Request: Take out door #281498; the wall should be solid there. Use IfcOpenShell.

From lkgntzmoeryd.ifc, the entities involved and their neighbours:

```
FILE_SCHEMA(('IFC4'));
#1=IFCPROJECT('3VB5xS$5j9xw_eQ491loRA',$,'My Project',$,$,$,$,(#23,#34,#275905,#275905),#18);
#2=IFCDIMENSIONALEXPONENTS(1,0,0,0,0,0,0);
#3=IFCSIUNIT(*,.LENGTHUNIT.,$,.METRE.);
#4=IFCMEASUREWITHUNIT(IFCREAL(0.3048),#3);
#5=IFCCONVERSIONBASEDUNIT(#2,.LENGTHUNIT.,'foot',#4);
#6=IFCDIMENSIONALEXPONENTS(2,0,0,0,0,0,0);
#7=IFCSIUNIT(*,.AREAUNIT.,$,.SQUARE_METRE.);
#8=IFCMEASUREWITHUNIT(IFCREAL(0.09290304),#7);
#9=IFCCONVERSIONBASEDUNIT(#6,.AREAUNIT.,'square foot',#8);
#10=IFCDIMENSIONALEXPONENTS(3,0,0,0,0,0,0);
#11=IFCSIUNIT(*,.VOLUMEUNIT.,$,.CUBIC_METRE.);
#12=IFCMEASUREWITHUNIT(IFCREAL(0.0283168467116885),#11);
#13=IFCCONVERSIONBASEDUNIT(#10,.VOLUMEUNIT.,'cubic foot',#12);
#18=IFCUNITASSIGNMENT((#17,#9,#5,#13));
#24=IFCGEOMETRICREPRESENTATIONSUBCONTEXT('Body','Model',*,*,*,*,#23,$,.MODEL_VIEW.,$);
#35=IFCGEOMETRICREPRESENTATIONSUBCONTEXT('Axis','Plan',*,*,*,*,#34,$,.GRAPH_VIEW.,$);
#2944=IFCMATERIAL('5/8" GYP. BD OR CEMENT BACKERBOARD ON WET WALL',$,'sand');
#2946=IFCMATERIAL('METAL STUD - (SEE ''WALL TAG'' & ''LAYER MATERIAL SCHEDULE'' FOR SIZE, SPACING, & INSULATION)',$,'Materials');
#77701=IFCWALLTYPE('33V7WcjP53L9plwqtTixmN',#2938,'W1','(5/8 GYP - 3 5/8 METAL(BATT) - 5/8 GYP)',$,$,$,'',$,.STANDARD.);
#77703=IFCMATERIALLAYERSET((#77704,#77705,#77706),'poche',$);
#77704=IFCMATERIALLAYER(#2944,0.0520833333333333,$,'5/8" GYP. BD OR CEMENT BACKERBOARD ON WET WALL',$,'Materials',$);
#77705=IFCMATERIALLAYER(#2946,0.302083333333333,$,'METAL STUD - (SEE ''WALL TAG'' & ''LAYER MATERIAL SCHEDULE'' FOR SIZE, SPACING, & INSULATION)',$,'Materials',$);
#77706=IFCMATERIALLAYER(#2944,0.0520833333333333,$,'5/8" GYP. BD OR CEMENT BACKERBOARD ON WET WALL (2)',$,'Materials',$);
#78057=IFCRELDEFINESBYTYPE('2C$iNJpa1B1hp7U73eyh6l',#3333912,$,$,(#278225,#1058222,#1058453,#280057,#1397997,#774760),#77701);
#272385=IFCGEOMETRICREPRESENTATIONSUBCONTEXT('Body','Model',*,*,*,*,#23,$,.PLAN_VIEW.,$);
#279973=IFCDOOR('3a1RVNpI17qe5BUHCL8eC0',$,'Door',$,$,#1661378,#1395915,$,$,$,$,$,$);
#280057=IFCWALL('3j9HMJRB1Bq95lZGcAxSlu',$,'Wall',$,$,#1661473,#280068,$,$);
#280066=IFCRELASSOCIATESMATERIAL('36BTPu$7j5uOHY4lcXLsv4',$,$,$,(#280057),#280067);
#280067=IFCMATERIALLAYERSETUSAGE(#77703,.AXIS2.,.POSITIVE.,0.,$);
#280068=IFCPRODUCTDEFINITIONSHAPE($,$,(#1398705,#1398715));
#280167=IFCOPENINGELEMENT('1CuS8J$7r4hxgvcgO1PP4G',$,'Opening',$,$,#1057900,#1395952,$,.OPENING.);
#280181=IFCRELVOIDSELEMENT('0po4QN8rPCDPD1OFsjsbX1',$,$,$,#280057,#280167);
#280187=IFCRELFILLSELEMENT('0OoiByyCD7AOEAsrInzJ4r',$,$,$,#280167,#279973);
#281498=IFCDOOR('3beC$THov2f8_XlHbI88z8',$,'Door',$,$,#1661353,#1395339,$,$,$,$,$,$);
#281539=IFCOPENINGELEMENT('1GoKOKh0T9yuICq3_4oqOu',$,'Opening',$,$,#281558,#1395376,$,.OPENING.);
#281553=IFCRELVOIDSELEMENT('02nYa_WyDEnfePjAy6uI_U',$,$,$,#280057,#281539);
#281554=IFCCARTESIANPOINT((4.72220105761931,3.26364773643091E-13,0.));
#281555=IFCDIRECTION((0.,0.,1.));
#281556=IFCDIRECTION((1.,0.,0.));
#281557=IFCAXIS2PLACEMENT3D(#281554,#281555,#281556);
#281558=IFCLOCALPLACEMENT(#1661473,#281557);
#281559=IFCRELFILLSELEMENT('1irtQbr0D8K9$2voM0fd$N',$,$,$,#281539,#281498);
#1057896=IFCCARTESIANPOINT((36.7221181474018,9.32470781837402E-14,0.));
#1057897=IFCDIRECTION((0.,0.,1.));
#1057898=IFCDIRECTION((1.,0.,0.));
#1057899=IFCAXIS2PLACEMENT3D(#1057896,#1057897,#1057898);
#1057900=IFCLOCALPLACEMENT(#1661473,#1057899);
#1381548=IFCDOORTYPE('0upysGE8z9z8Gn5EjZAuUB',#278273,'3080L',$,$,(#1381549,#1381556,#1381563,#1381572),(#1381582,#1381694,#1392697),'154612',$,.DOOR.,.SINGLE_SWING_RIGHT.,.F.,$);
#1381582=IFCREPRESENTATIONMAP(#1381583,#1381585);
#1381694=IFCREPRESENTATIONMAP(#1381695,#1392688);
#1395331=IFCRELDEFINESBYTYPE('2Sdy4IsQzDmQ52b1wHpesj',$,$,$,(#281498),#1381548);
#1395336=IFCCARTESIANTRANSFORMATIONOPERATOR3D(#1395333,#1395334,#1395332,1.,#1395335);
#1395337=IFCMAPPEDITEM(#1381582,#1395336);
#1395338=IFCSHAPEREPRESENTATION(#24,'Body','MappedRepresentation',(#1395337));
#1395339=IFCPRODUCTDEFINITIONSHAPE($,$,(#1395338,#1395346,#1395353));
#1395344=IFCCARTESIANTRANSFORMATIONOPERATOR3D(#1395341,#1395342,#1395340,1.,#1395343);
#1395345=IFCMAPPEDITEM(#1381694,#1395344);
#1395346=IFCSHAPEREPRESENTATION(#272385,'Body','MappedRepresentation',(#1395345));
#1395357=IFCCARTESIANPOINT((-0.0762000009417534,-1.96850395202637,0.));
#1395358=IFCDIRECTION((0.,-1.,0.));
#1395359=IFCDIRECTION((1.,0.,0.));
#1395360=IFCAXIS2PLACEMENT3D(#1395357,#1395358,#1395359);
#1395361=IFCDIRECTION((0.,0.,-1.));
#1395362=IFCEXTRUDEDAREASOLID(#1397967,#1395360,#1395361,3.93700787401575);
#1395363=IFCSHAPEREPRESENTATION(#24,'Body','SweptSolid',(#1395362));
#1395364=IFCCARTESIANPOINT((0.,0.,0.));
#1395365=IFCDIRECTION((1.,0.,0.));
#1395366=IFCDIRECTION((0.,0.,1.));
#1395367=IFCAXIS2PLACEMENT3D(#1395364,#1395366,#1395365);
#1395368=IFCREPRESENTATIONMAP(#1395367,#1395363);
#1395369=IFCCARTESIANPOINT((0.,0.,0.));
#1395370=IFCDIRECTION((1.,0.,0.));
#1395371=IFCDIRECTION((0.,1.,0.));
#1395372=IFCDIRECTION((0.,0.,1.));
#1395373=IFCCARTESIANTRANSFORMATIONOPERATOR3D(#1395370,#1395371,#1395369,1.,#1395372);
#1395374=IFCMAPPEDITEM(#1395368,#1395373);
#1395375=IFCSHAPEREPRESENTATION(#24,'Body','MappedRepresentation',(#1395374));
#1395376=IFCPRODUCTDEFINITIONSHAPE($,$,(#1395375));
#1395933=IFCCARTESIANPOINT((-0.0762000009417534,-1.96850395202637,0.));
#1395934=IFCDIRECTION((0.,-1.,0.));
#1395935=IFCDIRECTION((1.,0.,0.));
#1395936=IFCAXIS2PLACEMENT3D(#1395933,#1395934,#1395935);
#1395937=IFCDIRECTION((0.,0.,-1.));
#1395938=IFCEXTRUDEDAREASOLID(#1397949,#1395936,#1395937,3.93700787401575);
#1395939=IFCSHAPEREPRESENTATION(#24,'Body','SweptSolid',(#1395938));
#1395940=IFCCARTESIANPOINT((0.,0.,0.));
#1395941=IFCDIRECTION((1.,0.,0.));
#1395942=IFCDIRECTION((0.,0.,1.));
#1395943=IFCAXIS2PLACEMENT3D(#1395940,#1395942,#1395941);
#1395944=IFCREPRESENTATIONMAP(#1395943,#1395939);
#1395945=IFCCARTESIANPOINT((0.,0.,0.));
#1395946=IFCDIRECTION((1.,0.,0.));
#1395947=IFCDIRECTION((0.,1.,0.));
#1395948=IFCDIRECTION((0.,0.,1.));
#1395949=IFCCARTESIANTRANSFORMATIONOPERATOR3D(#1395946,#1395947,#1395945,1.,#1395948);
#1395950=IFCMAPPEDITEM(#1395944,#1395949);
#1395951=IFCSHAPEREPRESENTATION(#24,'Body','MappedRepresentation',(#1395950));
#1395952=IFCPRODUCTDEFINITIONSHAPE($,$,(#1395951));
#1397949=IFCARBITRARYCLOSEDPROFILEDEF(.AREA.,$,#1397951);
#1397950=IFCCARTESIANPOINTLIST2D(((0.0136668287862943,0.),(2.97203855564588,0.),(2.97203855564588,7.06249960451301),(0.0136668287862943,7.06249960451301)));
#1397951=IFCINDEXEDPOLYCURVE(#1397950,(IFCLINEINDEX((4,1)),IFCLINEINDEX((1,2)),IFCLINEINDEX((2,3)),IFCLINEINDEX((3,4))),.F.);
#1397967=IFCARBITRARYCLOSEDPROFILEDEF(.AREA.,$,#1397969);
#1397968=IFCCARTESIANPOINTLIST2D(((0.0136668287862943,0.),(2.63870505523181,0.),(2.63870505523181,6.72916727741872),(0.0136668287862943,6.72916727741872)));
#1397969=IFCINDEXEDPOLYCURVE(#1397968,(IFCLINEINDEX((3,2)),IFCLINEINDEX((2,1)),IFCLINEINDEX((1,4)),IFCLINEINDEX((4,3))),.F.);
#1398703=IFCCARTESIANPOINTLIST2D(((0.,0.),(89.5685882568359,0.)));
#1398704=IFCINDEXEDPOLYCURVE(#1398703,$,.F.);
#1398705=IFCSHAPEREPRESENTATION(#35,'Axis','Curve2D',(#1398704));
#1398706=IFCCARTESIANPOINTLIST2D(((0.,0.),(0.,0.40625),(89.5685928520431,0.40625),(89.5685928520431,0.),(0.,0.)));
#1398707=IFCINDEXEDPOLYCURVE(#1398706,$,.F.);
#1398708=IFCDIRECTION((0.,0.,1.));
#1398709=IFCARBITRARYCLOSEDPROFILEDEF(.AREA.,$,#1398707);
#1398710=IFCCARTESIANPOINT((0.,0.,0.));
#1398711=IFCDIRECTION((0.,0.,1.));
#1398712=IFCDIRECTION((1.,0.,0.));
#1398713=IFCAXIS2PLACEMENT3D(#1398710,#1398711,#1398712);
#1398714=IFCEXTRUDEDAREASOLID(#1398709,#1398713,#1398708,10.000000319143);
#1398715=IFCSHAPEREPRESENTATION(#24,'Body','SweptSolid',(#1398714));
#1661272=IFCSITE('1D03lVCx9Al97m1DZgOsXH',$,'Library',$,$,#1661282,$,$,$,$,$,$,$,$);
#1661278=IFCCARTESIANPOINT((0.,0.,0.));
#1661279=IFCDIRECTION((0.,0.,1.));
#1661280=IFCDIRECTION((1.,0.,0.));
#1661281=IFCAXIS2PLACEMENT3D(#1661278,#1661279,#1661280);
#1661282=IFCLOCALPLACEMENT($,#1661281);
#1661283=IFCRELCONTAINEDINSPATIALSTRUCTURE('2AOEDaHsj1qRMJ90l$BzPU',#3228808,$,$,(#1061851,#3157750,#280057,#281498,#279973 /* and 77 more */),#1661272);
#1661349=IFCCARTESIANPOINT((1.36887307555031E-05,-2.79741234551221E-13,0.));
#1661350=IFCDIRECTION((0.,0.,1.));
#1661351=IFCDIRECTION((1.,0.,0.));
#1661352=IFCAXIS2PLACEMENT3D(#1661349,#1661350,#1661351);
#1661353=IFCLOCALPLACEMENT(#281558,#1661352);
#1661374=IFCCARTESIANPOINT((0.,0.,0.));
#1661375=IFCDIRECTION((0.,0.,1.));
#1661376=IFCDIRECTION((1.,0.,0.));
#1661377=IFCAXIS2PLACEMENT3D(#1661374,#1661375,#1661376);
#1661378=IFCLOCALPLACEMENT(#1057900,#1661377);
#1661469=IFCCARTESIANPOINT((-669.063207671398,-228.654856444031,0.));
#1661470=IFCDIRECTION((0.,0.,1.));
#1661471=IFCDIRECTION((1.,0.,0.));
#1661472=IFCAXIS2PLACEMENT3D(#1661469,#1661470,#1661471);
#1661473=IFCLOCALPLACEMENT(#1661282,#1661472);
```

```python
import ifcopenshell
import ifcopenshell.api.feature
import ifcopenshell.api.root
import ifcopenshell.geom
import ifcopenshell.util.shape

model = ifcopenshell.open("lkgntzmoeryd.ifc")
settings = ifcopenshell.geom.settings()


def volume(element):
    """Net volume in cubic metres, openings subtracted."""
    shape = ifcopenshell.geom.create_shape(settings, element)
    return ifcopenshell.util.shape.get_volume(shape.geometry)


door = model.by_guid("3beC$THov2f8_XlHbI88z8")
opening = door.FillsVoids[0].RelatingOpeningElement
wall = opening.VoidsElements[0].RelatingBuildingElement
before = volume(wall)

ifcopenshell.api.root.remove_product(model, product=door)
ifcopenshell.api.feature.remove_feature(model, feature=opening)

after = volume(wall)

print(f"wall volume {before:.3f} -> {after:.3f} m3")

model.write("lkgntzmoeryd-out.ifc")
```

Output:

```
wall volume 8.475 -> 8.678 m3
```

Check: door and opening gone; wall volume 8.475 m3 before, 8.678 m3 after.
